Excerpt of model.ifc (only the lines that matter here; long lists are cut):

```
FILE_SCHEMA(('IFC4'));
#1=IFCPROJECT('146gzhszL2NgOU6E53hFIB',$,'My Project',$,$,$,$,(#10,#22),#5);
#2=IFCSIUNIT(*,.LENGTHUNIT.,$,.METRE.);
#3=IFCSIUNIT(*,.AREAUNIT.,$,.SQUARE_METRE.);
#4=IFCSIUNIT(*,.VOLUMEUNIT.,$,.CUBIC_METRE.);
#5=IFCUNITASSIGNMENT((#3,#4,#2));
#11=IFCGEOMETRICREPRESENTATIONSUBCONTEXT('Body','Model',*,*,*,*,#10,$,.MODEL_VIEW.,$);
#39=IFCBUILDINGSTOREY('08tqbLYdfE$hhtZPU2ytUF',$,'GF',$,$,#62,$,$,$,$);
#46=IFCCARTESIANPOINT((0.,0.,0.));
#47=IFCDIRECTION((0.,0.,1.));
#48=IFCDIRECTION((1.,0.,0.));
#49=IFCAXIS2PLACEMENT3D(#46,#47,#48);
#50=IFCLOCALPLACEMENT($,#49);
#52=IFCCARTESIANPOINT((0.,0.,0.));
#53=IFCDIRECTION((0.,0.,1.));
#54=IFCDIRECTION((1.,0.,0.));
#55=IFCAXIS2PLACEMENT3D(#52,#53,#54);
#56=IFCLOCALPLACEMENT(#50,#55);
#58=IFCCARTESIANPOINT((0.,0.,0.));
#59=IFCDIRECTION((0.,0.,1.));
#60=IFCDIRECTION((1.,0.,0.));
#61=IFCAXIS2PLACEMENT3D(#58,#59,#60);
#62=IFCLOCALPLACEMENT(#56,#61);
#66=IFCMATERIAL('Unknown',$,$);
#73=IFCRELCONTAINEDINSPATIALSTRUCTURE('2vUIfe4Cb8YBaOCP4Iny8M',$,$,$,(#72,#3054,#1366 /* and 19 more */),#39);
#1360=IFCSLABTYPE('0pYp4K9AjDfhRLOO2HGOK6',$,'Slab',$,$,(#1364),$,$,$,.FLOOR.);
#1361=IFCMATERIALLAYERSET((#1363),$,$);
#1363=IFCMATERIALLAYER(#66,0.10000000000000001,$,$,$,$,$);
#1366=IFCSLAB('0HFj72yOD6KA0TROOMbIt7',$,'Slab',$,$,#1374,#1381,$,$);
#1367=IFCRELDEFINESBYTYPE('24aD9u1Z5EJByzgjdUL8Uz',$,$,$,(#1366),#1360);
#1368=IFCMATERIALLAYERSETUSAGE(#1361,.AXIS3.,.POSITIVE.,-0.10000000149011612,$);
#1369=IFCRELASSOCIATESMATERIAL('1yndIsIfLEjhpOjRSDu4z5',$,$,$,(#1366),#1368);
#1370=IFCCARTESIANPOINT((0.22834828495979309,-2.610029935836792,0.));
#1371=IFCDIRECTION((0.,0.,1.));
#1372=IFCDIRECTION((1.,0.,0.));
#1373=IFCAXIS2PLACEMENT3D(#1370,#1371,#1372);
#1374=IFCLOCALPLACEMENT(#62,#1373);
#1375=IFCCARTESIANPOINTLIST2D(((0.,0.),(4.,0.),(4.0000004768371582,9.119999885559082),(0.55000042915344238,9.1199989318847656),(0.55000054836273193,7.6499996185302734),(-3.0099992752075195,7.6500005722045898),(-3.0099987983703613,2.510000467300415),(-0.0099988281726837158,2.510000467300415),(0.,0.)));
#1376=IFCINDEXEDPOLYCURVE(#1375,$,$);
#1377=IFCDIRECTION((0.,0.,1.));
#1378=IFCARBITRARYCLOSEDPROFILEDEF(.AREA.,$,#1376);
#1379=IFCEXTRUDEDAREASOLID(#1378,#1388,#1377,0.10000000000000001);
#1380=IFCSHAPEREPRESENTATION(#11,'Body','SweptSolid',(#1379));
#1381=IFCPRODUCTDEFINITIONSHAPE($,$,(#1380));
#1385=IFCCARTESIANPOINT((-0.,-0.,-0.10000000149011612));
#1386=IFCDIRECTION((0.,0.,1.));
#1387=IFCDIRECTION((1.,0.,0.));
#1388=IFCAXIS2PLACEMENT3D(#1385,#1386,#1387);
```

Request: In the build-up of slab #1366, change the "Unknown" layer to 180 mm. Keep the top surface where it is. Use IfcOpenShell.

```python
import ifcopenshell
import ifcopenshell.util.element
import ifcopenshell.util.representation

model = ifcopenshell.open("model.ifc")

layer_set = model.by_id(1361)
layer = next(l for l in layer_set.MaterialLayers if l.Material and l.Material.Name == "Unknown")
change = 0.18 - layer.LayerThickness
layer.LayerThickness += change

# Geometry does not follow the layer set by itself.
slabs = [e for e in ifcopenshell.util.element.get_elements_by_material(model, layer_set) if e.is_a("IfcSlab")]
for slab in sorted(slabs, key=lambda e: e.id()):
    body = ifcopenshell.util.representation.get_representation(slab, "Model", "Body")
    solid = body.Items[0]
    old_depth = solid.Depth
    solid.Depth += change
    # Extruded upwards: lower the start of the extrusion so the top stays.
    x, y, z = solid.Position.Location.Coordinates
    solid.Position.Location = model.createIfcCartesianPoint((x, y, z - change))
    print(slab.id(), f"{old_depth:g} -> {solid.Depth:g}")

# The layers are counted up from the underside, which has moved.
for usage in {ifcopenshell.util.element.get_material(slab) for slab in slabs}:
    usage.OffsetFromReferenceLine -= change

model.write("model_edited.ifc")
```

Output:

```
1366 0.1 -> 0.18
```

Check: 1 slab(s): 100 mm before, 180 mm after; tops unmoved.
